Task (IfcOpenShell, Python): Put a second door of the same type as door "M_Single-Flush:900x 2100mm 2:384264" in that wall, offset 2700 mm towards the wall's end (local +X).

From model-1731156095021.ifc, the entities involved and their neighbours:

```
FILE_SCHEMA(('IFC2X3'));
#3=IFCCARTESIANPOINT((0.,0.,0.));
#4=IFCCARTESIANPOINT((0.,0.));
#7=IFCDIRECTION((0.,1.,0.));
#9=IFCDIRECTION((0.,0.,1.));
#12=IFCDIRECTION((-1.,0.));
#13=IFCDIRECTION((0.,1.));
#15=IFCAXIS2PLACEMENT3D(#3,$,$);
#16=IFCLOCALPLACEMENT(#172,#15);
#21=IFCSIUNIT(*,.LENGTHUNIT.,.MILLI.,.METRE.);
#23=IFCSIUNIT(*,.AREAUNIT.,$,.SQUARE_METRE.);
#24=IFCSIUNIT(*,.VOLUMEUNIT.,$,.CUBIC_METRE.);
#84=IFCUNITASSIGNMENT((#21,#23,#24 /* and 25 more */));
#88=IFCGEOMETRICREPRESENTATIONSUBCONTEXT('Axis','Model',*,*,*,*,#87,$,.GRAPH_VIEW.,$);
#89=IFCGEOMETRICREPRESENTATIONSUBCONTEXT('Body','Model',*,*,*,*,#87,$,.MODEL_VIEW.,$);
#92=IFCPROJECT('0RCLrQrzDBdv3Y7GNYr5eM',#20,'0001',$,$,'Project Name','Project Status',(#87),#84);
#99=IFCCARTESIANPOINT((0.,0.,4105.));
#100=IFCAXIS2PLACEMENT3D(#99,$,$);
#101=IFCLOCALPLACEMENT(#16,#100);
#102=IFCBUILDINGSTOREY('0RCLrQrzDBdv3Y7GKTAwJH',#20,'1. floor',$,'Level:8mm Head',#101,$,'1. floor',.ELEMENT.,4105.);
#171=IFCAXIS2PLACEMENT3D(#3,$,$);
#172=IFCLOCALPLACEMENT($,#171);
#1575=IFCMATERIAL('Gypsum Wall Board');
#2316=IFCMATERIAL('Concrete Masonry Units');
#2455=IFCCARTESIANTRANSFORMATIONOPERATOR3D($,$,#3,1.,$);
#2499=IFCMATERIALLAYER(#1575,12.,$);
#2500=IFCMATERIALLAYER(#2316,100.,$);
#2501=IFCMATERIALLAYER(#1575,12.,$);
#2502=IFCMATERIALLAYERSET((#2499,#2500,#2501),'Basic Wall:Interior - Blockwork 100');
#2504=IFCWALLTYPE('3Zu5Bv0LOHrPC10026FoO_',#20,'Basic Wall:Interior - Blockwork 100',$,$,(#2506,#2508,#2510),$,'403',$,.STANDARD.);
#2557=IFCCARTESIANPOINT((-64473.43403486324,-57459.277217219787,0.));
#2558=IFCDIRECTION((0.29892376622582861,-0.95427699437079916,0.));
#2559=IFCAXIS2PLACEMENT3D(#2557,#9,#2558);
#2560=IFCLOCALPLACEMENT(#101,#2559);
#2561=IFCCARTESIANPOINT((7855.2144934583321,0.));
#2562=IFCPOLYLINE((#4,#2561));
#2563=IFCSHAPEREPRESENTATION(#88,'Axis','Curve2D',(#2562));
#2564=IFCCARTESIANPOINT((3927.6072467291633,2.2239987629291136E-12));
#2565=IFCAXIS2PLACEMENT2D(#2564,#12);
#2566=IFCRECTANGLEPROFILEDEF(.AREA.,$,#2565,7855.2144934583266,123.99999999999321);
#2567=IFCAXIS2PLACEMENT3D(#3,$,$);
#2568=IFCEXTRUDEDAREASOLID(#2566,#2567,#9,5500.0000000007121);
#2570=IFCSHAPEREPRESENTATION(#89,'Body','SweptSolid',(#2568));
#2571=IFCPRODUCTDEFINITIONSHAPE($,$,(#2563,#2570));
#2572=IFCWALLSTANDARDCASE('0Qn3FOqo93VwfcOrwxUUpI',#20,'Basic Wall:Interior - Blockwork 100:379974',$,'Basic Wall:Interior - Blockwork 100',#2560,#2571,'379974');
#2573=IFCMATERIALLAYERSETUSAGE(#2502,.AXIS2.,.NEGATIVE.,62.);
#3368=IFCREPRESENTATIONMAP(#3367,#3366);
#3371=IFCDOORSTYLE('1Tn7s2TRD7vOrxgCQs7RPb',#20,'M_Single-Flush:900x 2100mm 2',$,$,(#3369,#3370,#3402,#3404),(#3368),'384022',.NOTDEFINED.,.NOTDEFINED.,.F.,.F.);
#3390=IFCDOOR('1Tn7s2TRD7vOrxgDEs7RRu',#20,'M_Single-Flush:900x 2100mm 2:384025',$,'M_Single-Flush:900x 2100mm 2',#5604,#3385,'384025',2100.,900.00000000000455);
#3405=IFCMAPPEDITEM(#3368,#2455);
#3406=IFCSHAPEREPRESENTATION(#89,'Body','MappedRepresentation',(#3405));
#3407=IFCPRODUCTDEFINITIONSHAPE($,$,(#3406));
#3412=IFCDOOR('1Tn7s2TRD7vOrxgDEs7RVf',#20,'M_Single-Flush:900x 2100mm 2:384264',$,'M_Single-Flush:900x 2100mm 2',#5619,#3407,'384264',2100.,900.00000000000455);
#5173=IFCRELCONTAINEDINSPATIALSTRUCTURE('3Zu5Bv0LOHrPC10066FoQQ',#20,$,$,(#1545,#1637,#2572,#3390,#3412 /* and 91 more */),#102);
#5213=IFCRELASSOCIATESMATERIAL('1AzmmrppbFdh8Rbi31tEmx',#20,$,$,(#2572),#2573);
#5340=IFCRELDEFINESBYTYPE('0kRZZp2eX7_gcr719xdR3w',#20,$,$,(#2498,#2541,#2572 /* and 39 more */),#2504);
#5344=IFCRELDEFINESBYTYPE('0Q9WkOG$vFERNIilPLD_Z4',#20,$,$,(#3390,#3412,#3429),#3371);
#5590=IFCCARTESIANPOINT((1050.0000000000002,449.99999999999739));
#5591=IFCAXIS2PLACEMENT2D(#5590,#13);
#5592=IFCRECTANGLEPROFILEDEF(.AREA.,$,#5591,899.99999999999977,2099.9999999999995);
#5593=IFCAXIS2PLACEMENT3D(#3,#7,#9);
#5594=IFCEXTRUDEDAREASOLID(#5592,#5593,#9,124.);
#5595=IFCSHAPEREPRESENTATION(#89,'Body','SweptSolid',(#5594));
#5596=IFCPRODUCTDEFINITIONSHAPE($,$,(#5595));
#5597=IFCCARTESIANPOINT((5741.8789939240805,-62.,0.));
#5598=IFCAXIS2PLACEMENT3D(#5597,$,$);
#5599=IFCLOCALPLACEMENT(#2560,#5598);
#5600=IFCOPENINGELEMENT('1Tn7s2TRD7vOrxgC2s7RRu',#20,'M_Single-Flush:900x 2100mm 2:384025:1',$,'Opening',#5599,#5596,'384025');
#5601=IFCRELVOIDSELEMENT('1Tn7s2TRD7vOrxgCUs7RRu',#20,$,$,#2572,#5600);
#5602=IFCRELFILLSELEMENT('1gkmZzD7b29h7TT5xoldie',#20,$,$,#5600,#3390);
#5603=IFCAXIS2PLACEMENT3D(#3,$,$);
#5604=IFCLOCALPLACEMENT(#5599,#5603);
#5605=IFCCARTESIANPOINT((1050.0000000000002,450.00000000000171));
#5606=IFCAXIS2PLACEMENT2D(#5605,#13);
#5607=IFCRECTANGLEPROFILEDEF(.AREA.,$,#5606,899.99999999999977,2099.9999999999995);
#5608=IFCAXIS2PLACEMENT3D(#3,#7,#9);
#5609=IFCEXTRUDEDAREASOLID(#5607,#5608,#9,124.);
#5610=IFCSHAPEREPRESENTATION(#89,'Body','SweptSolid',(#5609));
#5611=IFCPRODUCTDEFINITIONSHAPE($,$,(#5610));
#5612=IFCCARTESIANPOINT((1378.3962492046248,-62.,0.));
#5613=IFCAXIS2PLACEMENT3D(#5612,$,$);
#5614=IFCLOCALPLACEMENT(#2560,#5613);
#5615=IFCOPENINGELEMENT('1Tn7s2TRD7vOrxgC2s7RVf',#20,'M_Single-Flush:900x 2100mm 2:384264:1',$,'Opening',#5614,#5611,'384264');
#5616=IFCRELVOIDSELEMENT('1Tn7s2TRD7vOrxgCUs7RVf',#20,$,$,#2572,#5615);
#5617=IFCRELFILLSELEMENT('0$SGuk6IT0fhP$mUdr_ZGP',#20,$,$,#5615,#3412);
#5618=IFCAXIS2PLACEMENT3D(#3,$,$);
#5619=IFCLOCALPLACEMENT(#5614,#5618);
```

```python
import ifcopenshell
import ifcopenshell.api.feature
import ifcopenshell.api.geometry
import ifcopenshell.api.root
import ifcopenshell.geom
import ifcopenshell.util.element
import ifcopenshell.util.placement
import ifcopenshell.util.shape

model = ifcopenshell.open("model-1731156095021.ifc")
settings = ifcopenshell.geom.settings()


def volume(element):
    """Net volume in cubic metres, openings subtracted."""
    shape = ifcopenshell.geom.create_shape(settings, element)
    return ifcopenshell.util.shape.get_volume(shape.geometry)


def reuse_history(source, copy):
    """copy_class also copies each property set's owner history, people and application; keep the originals."""
    for rel in copy.IsDefinedBy:
        if rel.is_a("IfcRelDefinesByProperties") and (history := rel.RelatingPropertyDefinition.OwnerHistory):
            rel.RelatingPropertyDefinition.OwnerHistory = source.OwnerHistory
            ifcopenshell.util.element.remove_deep2(model, history)


door = model.by_guid("1Tn7s2TRD7vOrxgDEs7RVf")
opening = door.FillsVoids[0].RelatingOpeningElement
wall = opening.VoidsElements[0].RelatingBuildingElement
before = volume(wall)
shift = ifcopenshell.util.placement.get_local_placement(wall.ObjectPlacement)[:3, 0] * 2700.0

# copy_class copies the void relationship, type, container and properties, but no geometry.
new_opening = ifcopenshell.api.root.copy_class(model, product=opening)
new_opening.Representation = ifcopenshell.util.element.copy_deep(
    model, opening.Representation, exclude=["IfcGeometricRepresentationContext", "IfcRepresentationMap"]
)
new_opening.Name = "M_Single-Flush:900x 2100mm 2"
new_opening.Tag = None
new_door = ifcopenshell.api.root.copy_class(model, product=door)
new_door.Representation = ifcopenshell.util.element.copy_deep(
    model, door.Representation, exclude=["IfcGeometricRepresentationContext", "IfcRepresentationMap"]
)
new_door.Name = "M_Single-Flush:900x 2100mm 2"
new_door.Tag = None
reuse_history(door, new_door)
fills = ifcopenshell.api.feature.add_filling(model, opening=new_opening, element=new_door)
fills.OwnerHistory = new_door.OwnerHistory  # required in IFC2X3

for old, new in ((opening, new_opening), (door, new_door)):
    matrix = ifcopenshell.util.placement.get_local_placement(old.ObjectPlacement)
    matrix[:3, 3] += shift
    ifcopenshell.api.geometry.edit_object_placement(model, product=new, matrix=matrix, is_si=False)

after = volume(wall)

print(f"wall volume {before:.3f} -> {after:.3f} m3")

model.write("model-1731156095021_edited.ifc")
```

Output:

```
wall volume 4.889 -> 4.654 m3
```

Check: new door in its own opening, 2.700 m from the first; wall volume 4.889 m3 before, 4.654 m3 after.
